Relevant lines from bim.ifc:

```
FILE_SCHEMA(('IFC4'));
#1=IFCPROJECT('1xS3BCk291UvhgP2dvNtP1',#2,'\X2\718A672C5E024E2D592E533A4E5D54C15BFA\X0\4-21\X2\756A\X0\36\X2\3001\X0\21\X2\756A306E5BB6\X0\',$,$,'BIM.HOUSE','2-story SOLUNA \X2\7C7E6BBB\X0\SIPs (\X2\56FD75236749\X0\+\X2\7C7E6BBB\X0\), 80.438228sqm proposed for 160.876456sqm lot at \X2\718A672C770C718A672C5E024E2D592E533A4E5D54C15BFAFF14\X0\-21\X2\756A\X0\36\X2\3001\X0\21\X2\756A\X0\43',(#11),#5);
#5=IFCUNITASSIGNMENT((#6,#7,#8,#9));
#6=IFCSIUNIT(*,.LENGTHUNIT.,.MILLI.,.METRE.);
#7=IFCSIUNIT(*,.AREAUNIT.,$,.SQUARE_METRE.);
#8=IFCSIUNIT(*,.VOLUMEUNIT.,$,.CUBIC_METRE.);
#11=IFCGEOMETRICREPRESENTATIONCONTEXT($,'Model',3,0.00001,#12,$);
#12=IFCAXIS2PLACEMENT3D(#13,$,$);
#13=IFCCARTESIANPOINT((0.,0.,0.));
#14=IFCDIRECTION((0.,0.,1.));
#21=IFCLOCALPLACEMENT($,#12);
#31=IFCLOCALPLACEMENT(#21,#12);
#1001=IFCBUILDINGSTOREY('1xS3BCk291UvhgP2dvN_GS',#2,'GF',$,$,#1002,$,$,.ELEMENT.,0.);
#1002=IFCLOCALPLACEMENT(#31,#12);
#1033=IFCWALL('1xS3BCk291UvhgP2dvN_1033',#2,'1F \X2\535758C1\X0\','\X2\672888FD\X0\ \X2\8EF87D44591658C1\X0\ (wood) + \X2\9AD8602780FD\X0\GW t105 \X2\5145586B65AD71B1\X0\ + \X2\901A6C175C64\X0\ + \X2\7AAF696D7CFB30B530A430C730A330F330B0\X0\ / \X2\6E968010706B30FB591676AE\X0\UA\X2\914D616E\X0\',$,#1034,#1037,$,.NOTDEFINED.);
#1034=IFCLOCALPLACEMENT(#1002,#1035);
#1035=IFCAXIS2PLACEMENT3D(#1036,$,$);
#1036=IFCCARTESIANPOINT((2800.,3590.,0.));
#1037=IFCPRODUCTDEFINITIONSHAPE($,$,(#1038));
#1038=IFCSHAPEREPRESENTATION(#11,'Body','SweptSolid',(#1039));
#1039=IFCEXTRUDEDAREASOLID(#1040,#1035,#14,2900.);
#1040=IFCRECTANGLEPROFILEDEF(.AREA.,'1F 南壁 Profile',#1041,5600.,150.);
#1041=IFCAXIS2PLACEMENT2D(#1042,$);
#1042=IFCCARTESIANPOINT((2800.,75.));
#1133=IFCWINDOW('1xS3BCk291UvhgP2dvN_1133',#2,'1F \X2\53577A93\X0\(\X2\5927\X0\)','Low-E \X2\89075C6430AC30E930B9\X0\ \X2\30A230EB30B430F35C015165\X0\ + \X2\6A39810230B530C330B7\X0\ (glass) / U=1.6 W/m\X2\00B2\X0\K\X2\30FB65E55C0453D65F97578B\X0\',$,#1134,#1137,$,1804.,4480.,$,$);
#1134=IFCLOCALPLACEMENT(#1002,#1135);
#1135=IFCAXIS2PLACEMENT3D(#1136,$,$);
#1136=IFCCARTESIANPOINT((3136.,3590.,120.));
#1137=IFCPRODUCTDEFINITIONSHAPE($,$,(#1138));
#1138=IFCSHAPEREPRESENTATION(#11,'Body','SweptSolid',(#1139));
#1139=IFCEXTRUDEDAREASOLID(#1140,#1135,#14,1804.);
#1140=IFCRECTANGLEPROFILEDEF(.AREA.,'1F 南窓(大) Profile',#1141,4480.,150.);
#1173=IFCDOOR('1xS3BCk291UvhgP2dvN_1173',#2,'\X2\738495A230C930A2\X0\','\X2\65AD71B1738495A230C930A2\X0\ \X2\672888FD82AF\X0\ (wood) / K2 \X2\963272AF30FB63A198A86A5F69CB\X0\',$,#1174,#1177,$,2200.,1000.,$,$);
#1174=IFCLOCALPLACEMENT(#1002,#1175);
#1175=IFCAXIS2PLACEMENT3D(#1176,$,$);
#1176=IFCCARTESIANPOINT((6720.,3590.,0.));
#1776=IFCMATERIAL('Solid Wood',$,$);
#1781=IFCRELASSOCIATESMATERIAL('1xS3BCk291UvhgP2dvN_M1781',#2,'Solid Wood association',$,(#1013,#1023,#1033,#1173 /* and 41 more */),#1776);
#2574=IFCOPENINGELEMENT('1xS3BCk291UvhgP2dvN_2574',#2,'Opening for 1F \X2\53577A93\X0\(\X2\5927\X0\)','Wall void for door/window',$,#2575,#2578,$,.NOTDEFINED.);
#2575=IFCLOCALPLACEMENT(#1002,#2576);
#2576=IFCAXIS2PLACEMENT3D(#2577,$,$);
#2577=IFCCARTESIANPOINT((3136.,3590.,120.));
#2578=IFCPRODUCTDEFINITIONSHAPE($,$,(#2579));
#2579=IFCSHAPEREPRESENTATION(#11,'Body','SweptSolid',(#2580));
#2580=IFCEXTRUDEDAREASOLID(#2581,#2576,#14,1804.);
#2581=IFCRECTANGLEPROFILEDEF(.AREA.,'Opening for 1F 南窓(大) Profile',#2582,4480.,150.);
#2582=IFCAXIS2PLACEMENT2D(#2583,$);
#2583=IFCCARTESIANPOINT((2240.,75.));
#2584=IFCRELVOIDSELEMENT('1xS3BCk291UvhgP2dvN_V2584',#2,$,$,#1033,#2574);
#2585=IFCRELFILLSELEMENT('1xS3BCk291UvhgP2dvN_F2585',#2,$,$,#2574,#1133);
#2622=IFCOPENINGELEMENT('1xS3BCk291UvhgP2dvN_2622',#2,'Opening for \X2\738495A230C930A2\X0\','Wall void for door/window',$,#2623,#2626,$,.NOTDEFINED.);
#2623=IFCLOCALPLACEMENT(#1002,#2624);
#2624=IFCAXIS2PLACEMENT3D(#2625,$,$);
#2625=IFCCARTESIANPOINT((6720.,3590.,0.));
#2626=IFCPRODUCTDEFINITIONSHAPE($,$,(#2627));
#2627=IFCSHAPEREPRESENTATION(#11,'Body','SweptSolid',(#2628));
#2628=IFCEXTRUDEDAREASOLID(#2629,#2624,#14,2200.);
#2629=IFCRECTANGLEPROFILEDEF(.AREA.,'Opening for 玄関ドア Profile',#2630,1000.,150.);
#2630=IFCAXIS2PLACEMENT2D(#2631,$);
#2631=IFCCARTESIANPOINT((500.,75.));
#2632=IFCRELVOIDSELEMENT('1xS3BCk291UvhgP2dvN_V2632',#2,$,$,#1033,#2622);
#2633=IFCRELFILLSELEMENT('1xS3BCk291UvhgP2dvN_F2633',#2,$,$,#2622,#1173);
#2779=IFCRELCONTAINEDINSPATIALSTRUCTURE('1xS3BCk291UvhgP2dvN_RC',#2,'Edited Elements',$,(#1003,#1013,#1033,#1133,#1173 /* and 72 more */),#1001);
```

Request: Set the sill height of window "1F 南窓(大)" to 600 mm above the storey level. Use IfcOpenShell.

```python
import numpy as np
import ifcopenshell
import ifcopenshell.api.geometry
import ifcopenshell.geom
import ifcopenshell.util.element
import ifcopenshell.util.placement
import ifcopenshell.util.shape
import ifcopenshell.util.unit

model = ifcopenshell.open("bim.ifc")
unit_scale = ifcopenshell.util.unit.calculate_unit_scale(model)

window = model.by_guid("1xS3BCk291UvhgP2dvN_1133")
opening = window.FillsVoids[0].RelatingOpeningElement
storey = ifcopenshell.util.element.get_container(window, ifc_class="IfcBuildingStorey")
level = ifcopenshell.util.placement.get_local_placement(storey.ObjectPlacement)[2, 3]

# The opening's origin need not be at the sill, so measure its lowest point.
shape = ifcopenshell.geom.create_shape(ifcopenshell.geom.settings(), opening)
bottom = ifcopenshell.util.shape.get_shape_bottom_elevation(shape, shape.geometry) / unit_scale
dz = level + 0.6 / unit_scale - bottom

shift = np.array([0.0, 0.0, dz])
# The window is not placed relative to its opening, so move both.
for product in (opening, window):
    matrix = ifcopenshell.util.placement.get_local_placement(product.ObjectPlacement)
    matrix[:3, 3] += shift
    ifcopenshell.api.geometry.edit_object_placement(model, product=product, matrix=matrix, is_si=False)

print(f"moved by {dz * unit_scale:+.3f} m")

model.write("bim_v2.ifc")
```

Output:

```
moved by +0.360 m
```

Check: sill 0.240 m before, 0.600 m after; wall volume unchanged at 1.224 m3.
